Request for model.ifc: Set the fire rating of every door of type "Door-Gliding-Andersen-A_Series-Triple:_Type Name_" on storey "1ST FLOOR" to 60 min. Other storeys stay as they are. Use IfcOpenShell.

First a look at what the model holds.

```python
import ifcopenshell
import ifcopenshell.util.element

model = ifcopenshell.open("model.ifc")
print(model.schema)
storey = next(s for s in model.by_type("IfcBuildingStorey") if s.Name == "1ST FLOOR")
doors = [e for e in ifcopenshell.util.element.get_decomposition(storey) if e.is_a("IfcDoor")]
seen = {}
for e in doors:
    element_type = ifcopenshell.util.element.get_type(e)
    key = (element_type.Name if element_type != e and element_type else None, ifcopenshell.util.element.get_pset(e, "Pset_DoorCommon", "FireRating"))
    seen[key] = seen.get(key, 0) + 1
for (name, value), count in sorted(seen.items(), key=str):
    print(count, "x", name, "|", value)
```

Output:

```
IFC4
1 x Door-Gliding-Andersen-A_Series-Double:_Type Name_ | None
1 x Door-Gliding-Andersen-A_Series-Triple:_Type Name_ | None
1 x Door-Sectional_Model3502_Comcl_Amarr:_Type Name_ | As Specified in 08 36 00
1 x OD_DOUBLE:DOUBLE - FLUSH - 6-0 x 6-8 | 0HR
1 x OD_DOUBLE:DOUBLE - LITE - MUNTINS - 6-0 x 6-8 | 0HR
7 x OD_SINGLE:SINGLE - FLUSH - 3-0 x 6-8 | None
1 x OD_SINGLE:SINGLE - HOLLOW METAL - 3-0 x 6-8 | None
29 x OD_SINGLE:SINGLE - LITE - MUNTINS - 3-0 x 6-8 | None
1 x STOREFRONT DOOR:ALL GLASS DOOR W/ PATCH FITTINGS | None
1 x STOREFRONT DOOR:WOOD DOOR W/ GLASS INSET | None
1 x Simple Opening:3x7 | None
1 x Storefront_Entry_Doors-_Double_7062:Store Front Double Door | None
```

```python
import ifcopenshell
import ifcopenshell.api.pset
import ifcopenshell.util.element

model = ifcopenshell.open("model.ifc")

storey = next(s for s in model.by_type("IfcBuildingStorey") if s.Name == "1ST FLOOR")
doors = [e for e in ifcopenshell.util.element.get_decomposition(storey) if e.is_a("IfcDoor")]

count = 0
for e in doors:
    element_type = ifcopenshell.util.element.get_type(e)
    if element_type in (None, e) or element_type.Name != "Door-Gliding-Andersen-A_Series-Triple:_Type Name_":
        continue
    # add_pset returns the element's existing set when there is one.
    pset = ifcopenshell.api.pset.add_pset(model, product=e, name="Pset_DoorCommon")
    ifcopenshell.api.pset.edit_pset(model, pset=pset, properties={"FireRating": "60 min"})
    count += 1

print(count, "doors updated")

model.write("model_updated.ifc")
```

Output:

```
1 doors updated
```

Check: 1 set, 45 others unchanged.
